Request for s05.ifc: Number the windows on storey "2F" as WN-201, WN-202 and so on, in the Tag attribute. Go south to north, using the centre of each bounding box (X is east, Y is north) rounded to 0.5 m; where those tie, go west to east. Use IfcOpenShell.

First a look at what the model holds.

```python
import ifcopenshell
import ifcopenshell.util.element
import ifcopenshell.util.placement

model = ifcopenshell.open("s05.ifc")
print(model.schema)
storey = next(s for s in model.by_type("IfcBuildingStorey") if s.Name == "2F")
windows = [e for e in ifcopenshell.util.element.get_decomposition(storey) if e.is_a("IfcWindow")]
for e in sorted(windows, key=lambda e: e.id()):
    origin = ifcopenshell.util.placement.get_local_placement(e.ObjectPlacement)[:3, 3]
    print(e.id(), e.Tag, e.Name, origin.round(2) + 0.0, sep=" | ")
```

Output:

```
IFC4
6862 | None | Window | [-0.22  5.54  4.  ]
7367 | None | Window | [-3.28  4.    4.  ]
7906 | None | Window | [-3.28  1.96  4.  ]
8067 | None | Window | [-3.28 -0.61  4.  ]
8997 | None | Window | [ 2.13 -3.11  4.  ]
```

```python
import ifcopenshell
import ifcopenshell.geom
import ifcopenshell.util.element
import ifcopenshell.util.shape

model = ifcopenshell.open("s05.ifc")
settings = ifcopenshell.geom.settings()
settings.set("use-world-coords", True)


def centre(element):
    shape = ifcopenshell.geom.create_shape(settings, element)
    return ifcopenshell.util.shape.get_bbox_centroid(shape.geometry)


storey = next(s for s in model.by_type("IfcBuildingStorey") if s.Name == "2F")
windows = [e for e in ifcopenshell.util.element.get_decomposition(storey) if e.is_a("IfcWindow")]

# Insertion points can sit at a corner or the storey origin, so sort by the geometry (in metres).
centres = {e: centre(e) for e in windows}
windows.sort(key=lambda e: (round(centres[e][1] / 0.5), centres[e][0]))

for i, e in enumerate(windows, start=1):
    number = f"WN-2{i:02d}"
    e.Tag = number
    print(e.id(), number)

model.write("s05_rev.ifc")
```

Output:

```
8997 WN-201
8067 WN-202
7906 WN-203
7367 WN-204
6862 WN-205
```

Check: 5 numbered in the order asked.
